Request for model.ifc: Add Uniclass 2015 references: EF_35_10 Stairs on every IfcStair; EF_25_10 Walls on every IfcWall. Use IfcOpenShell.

First a look at what the model holds.

```python
import ifcopenshell

model = ifcopenshell.open("model.ifc")
print(model.schema)
print("classifications:", [c.Name for c in model.by_type("IfcClassification")])
for ifc_class in ("IfcDoor", "IfcRoof", "IfcStair", "IfcWall", "IfcWindow"):
    print(ifc_class, len(model.by_type(ifc_class)))
```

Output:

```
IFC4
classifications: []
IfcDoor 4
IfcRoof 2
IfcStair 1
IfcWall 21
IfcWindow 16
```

```python
import ifcopenshell
import ifcopenshell.api.classification

model = ifcopenshell.open("model.ifc")

system = ifcopenshell.api.classification.add_classification(model, classification="Uniclass 2015")

codes = {
    "IfcStair": ("EF_35_10", "Stairs"),
    "IfcWall": ("EF_25_10", "Walls"),
}
for ifc_class, (code, name) in codes.items():
    products = model.by_type(ifc_class)
    ifcopenshell.api.classification.add_reference(
        model, products=products, classification=system, identification=code, name=name
    )
    print(code, len(products))

model.write("model_v2.ifc")
```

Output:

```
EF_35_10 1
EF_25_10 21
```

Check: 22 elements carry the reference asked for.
